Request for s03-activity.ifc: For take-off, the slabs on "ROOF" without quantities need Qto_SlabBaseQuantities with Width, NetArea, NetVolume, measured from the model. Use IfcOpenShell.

First a look at what the model holds.

```python
import ifcopenshell
import ifcopenshell.util.element
import ifcopenshell.util.unit

model = ifcopenshell.open("s03-activity.ifc")
print(model.schema)
for unit_type in ("LENGTHUNIT", "AREAUNIT", "VOLUMEUNIT"):
    print(unit_type, ifcopenshell.util.unit.calculate_unit_scale(model, unit_type))
storey = next(s for s in model.by_type("IfcBuildingStorey") if s.Name == "ROOF")
slabs = [e for e in ifcopenshell.util.element.get_decomposition(storey) if e.is_a("IfcSlab")]
for e in sorted(slabs, key=lambda e: e.id()):
    print(e.id(), e.is_a(), e.Name, list(ifcopenshell.util.element.get_psets(e, qtos_only=True)), sep=" | ")
```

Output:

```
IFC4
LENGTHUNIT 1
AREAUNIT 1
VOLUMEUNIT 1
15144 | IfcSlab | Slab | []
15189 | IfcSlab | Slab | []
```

```python
import ifcopenshell
import ifcopenshell.api.pset
import ifcopenshell.geom
import ifcopenshell.util.element
import ifcopenshell.util.shape
import ifcopenshell.util.unit

model = ifcopenshell.open("s03-activity.ifc")
unit_scale = ifcopenshell.util.unit.calculate_unit_scale(model)
area_scale = ifcopenshell.util.unit.calculate_unit_scale(model, "AREAUNIT")
volume_scale = ifcopenshell.util.unit.calculate_unit_scale(model, "VOLUMEUNIT")
settings = ifcopenshell.geom.settings()

storey = next(s for s in model.by_type("IfcBuildingStorey") if s.Name == "ROOF")
slabs = [e for e in ifcopenshell.util.element.get_decomposition(storey) if e.is_a("IfcSlab")]

for e in sorted(slabs, key=lambda e: e.id()):
    if ifcopenshell.util.element.get_psets(e, qtos_only=True, should_inherit=False):
        continue
    # Geometry comes back in metres, in the element's own axes.
    shape = ifcopenshell.geom.create_shape(settings, e)
    values = {
        "Width": ifcopenshell.util.shape.get_z(shape.geometry) / unit_scale,
        "NetArea": ifcopenshell.util.shape.get_footprint_area(shape.geometry) / area_scale,
        "NetVolume": ifcopenshell.util.shape.get_volume(shape.geometry) / volume_scale,
    }
    qto = ifcopenshell.api.pset.add_qto(model, product=e, name="Qto_SlabBaseQuantities")
    ifcopenshell.api.pset.edit_qto(model, qto=qto, properties=values)
    print(e.id(), {k: round(v, 3) for k, v in values.items()})

model.write("s03-activity-out.ifc")
```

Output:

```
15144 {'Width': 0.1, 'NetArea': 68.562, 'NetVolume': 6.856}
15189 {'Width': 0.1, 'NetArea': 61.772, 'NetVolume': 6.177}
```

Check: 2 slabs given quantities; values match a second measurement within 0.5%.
